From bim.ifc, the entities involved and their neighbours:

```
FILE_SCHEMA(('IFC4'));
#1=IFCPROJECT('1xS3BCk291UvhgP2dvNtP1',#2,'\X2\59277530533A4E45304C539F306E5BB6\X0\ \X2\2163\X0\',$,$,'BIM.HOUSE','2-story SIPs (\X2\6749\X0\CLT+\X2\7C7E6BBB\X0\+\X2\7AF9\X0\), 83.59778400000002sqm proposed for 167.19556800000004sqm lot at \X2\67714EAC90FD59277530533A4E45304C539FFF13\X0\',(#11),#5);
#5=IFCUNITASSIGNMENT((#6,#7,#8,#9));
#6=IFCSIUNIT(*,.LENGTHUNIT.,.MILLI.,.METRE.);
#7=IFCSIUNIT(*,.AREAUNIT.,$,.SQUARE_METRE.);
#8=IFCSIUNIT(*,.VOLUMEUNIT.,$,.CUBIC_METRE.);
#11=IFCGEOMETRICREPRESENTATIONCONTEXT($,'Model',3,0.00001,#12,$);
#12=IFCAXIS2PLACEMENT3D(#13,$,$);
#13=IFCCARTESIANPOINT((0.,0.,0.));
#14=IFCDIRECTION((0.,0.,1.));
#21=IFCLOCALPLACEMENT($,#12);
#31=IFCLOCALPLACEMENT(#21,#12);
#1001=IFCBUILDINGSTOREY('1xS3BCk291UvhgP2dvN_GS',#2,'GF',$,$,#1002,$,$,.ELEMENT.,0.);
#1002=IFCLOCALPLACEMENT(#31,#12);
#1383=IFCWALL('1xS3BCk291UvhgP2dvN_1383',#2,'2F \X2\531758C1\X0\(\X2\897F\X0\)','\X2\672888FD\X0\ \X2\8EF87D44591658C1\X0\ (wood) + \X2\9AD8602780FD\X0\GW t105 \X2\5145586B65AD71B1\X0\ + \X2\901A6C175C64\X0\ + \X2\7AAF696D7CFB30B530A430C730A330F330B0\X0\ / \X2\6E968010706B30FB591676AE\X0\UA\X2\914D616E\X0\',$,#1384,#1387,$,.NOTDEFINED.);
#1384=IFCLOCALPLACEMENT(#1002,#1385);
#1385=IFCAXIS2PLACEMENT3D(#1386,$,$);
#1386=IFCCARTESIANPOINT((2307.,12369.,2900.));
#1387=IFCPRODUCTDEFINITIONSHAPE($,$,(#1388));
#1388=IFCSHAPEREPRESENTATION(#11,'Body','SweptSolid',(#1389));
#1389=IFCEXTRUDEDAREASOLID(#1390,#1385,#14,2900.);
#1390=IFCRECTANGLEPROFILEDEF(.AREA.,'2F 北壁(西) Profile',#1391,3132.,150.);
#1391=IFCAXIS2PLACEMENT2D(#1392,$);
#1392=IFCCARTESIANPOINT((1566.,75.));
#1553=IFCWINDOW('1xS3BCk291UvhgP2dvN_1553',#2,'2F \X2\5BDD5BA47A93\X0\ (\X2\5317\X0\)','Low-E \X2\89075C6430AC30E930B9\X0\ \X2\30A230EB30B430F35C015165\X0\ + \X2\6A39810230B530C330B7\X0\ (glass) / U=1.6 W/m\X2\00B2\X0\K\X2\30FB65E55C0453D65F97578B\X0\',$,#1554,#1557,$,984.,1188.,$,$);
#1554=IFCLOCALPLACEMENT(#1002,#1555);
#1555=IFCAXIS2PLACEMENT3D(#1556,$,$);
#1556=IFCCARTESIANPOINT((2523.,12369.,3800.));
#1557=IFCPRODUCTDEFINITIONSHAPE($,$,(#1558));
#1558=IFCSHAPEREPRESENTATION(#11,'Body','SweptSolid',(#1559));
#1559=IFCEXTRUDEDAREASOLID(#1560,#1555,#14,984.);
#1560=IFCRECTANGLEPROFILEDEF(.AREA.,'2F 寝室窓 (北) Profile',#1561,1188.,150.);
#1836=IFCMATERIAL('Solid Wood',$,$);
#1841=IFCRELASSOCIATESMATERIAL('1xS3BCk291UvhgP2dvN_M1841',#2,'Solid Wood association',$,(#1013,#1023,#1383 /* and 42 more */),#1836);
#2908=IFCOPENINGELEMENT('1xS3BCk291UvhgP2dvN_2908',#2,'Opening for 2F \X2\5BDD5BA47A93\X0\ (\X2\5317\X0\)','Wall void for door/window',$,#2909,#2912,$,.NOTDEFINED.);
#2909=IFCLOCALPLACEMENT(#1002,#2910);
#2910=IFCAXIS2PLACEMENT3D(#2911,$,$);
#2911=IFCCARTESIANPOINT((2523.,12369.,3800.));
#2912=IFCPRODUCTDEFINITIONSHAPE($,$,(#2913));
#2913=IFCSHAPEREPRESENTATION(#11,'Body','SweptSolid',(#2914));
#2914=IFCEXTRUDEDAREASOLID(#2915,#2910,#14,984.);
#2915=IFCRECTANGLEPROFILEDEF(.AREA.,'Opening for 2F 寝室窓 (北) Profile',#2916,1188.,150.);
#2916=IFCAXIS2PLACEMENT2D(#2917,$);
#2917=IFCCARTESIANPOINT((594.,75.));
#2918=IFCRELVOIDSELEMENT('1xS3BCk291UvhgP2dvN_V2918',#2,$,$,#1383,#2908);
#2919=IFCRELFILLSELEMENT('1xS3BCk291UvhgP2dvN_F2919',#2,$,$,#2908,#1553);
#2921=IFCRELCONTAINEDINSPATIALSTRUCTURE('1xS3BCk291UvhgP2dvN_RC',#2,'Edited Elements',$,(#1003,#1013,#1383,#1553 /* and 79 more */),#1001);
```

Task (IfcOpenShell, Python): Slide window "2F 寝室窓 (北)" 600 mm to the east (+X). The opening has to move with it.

```python
import ifcopenshell
import ifcopenshell.api.geometry
import ifcopenshell.util.placement

model = ifcopenshell.open("bim.ifc")

window = model.by_guid("1xS3BCk291UvhgP2dvN_1553")
opening = window.FillsVoids[0].RelatingOpeningElement
wall = opening.VoidsElements[0].RelatingBuildingElement

wall_matrix = ifcopenshell.util.placement.get_local_placement(wall.ObjectPlacement)
shift = wall_matrix[:3, 0] * 600.0
before = ifcopenshell.util.placement.get_local_placement(window.ObjectPlacement)[:3, 3].copy()

# The window is not placed relative to its opening, so move both.
for product in (opening, window):
    matrix = ifcopenshell.util.placement.get_local_placement(product.ObjectPlacement)
    matrix[:3, 3] += shift
    ifcopenshell.api.geometry.edit_object_placement(model, product=product, matrix=matrix, is_si=False)

after = ifcopenshell.util.placement.get_local_placement(window.ObjectPlacement)[:3, 3]
print("window moved by", (after - before).round(3) + 0.0)

model.write("bim_updated.ifc")
```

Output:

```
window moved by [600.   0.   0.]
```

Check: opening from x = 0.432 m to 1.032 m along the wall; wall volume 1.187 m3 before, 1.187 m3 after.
